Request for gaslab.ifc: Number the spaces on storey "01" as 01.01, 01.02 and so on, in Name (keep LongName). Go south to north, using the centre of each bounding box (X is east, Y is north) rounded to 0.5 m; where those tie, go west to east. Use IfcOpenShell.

First a look at what the model holds.

```python
import ifcopenshell
import ifcopenshell.util.element
import ifcopenshell.util.placement

model = ifcopenshell.open("gaslab.ifc")
print(model.schema)
storey = next(s for s in model.by_type("IfcBuildingStorey") if s.Name == "01")
spaces = [e for e in ifcopenshell.util.element.get_decomposition(storey) if e.is_a("IfcSpace")]
for e in sorted(spaces, key=lambda e: e.id()):
    origin = ifcopenshell.util.placement.get_local_placement(e.ObjectPlacement)[:3, 3]
    print(e.id(), e.Name, e.LongName, origin.round(2) + 0.0, sep=" | ")
```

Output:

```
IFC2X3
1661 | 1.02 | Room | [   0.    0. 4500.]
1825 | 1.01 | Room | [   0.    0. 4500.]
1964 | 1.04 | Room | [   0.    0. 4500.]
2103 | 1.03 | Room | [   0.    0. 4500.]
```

```python
import ifcopenshell
import ifcopenshell.geom
import ifcopenshell.util.element
import ifcopenshell.util.shape

model = ifcopenshell.open("gaslab.ifc")
settings = ifcopenshell.geom.settings()
settings.set("use-world-coords", True)


def centre(element):
    shape = ifcopenshell.geom.create_shape(settings, element)
    return ifcopenshell.util.shape.get_bbox_centroid(shape.geometry)


storey = next(s for s in model.by_type("IfcBuildingStorey") if s.Name == "01")
spaces = [e for e in ifcopenshell.util.element.get_decomposition(storey) if e.is_a("IfcSpace")]

# Insertion points can sit at a corner or the storey origin, so sort by the geometry (in metres).
centres = {e: centre(e) for e in spaces}
spaces.sort(key=lambda e: (round(centres[e][1] / 0.5), centres[e][0]))

for i, e in enumerate(spaces, start=1):
    number = f"01.{i:02d}"
    e.Name = number
    print(e.id(), number)

model.write("gaslab_updated.ifc")
```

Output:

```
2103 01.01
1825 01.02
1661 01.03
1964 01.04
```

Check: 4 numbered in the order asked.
